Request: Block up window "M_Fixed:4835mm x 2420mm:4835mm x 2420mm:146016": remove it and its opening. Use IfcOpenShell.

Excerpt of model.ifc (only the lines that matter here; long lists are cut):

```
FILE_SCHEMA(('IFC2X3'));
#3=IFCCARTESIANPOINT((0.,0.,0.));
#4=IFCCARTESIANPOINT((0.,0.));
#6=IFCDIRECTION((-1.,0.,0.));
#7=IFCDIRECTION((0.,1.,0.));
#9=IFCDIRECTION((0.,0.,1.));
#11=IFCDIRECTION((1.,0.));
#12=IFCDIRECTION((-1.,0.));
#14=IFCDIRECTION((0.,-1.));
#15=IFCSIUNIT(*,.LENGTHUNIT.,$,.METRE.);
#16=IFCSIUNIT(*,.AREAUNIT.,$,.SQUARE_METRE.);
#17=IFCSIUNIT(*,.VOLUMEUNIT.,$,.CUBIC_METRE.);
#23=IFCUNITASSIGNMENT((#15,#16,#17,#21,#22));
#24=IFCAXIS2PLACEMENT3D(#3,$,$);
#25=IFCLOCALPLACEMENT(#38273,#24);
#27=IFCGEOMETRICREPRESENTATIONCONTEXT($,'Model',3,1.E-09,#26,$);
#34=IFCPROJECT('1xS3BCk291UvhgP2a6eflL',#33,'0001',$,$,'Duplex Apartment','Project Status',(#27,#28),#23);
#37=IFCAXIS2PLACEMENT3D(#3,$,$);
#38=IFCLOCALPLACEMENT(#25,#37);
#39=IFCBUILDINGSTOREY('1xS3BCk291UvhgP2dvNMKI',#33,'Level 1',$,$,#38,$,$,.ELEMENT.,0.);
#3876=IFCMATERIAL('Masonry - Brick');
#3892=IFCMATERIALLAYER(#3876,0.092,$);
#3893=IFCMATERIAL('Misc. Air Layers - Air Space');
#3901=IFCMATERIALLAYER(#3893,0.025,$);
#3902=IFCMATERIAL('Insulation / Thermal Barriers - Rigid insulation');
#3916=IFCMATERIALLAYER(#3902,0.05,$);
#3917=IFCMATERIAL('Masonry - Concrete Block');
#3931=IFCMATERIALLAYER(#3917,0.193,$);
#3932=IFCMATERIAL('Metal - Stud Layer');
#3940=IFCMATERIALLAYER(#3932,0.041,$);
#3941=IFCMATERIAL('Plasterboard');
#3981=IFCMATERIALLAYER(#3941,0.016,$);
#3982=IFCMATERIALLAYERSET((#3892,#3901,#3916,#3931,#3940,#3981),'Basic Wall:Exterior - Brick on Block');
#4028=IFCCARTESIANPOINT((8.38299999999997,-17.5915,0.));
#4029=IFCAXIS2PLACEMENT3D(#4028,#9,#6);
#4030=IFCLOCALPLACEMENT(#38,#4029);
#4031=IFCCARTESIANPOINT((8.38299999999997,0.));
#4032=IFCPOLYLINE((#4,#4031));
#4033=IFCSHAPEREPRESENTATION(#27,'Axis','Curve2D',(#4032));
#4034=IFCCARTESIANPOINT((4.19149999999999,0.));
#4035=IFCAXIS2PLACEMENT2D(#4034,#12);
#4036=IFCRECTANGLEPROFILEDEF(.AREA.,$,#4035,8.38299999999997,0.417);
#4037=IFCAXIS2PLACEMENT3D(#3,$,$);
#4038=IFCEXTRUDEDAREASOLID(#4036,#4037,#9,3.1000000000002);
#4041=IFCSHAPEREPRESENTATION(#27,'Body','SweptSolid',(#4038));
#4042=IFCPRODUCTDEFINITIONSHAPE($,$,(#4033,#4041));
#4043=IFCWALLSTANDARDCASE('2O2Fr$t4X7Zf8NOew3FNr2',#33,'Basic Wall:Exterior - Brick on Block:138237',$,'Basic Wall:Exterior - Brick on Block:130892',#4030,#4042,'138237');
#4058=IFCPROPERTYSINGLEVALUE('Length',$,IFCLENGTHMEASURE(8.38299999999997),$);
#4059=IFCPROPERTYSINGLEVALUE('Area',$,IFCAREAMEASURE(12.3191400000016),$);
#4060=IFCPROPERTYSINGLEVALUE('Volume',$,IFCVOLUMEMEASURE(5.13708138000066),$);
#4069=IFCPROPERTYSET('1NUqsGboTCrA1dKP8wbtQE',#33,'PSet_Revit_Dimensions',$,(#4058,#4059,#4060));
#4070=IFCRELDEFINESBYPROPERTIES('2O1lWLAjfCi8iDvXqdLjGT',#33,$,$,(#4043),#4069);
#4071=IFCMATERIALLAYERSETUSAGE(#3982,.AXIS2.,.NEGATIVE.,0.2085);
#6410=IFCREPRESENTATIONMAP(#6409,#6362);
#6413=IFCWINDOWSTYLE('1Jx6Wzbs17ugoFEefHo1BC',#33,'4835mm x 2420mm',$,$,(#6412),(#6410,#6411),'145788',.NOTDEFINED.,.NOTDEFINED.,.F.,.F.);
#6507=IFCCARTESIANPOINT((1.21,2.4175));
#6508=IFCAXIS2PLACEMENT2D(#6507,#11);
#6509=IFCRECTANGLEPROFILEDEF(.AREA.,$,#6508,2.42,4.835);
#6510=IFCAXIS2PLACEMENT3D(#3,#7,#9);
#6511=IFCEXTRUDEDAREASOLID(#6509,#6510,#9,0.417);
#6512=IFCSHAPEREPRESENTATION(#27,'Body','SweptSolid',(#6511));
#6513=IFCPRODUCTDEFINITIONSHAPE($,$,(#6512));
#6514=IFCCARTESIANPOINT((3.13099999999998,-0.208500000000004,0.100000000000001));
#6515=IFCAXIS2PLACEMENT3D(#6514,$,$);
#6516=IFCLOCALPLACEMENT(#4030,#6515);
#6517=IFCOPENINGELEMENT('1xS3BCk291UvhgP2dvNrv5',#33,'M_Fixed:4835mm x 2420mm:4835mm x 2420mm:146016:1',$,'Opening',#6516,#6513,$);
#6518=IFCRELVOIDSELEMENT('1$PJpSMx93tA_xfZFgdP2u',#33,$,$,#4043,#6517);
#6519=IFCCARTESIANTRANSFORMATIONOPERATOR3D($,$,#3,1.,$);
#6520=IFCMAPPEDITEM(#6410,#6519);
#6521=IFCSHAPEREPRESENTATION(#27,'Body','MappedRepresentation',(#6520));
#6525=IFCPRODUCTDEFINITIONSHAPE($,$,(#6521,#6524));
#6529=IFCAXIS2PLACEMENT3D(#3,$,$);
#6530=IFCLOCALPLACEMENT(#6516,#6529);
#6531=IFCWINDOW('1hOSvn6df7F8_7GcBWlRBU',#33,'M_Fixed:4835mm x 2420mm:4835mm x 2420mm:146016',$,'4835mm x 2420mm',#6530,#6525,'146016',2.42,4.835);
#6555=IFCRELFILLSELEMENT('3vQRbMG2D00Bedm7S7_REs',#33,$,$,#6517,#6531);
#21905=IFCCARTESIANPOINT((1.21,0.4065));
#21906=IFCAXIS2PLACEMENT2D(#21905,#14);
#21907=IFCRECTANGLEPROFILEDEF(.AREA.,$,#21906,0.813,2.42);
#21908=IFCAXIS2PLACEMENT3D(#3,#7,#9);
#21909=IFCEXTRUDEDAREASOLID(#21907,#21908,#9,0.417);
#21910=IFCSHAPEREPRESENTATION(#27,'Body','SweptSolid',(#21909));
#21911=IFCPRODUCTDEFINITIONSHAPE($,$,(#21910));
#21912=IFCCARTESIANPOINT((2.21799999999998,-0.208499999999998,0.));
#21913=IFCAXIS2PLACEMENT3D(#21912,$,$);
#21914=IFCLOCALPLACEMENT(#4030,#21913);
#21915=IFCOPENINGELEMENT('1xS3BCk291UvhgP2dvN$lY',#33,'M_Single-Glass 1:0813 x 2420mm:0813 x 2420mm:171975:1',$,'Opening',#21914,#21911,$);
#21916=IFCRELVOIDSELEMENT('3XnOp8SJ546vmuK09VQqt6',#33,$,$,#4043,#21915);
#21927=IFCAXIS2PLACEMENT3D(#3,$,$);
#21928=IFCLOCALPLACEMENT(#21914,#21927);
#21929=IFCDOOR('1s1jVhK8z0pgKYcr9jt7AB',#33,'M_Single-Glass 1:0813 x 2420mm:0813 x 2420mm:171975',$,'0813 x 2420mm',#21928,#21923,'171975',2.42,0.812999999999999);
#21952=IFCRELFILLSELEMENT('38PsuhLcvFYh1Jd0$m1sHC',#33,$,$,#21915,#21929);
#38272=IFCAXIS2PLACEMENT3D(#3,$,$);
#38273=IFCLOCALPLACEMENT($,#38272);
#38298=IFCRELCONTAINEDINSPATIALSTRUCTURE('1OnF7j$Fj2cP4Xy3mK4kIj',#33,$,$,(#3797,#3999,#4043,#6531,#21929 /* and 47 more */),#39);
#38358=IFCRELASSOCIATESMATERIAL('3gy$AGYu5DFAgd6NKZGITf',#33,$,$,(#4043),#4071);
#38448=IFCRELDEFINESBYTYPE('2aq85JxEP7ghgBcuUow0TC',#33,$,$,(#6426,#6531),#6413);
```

```python
import ifcopenshell
import ifcopenshell.api.feature
import ifcopenshell.api.pset
import ifcopenshell.api.root
import ifcopenshell.geom
import ifcopenshell.util.element
import ifcopenshell.util.shape
import ifcopenshell.util.unit

model = ifcopenshell.open("model.ifc")
area_scale = ifcopenshell.util.unit.calculate_unit_scale(model, "AREAUNIT")
volume_scale = ifcopenshell.util.unit.calculate_unit_scale(model, "VOLUMEUNIT")
settings = ifcopenshell.geom.settings()


def volume(element):
    """Net volume in cubic metres, openings subtracted."""
    shape = ifcopenshell.geom.create_shape(settings, element)
    return ifcopenshell.util.shape.get_volume(shape.geometry)


window = model.by_guid("1hOSvn6df7F8_7GcBWlRBU")
opening = window.FillsVoids[0].RelatingOpeningElement
wall = opening.VoidsElements[0].RelatingBuildingElement
before = volume(wall)

ifcopenshell.api.root.remove_product(model, product=window)
ifcopenshell.api.feature.remove_feature(model, feature=opening)

after = volume(wall)
thickness = 0.417  # wall thickness in metres

# Update the wall's stored quantities.
pset = model.by_id(ifcopenshell.util.element.get_pset(wall, "PSet_Revit_Dimensions", should_inherit=False)["id"])
ifcopenshell.api.pset.edit_pset(model, pset=pset, properties={
    "Area": model.create_entity("IfcAreaMeasure", after / thickness / area_scale),
    "Volume": model.create_entity("IfcVolumeMeasure", after / volume_scale),
})

print(f"wall volume {before:.3f} -> {after:.3f} m3")

model.write("model-out.ifc")
```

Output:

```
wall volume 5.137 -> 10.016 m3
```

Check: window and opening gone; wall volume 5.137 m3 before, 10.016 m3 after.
